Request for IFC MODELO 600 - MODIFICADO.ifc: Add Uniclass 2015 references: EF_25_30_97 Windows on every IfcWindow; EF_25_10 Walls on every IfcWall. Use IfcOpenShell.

First a look at what the model holds.

```python
import ifcopenshell

model = ifcopenshell.open("IFC MODELO 600 - MODIFICADO.ifc")
print(model.schema)
print("classifications:", [c.Name for c in model.by_type("IfcClassification")])
for ifc_class in ("IfcDoor", "IfcRoof", "IfcStair", "IfcWall", "IfcWindow"):
    print(ifc_class, len(model.by_type(ifc_class)))
```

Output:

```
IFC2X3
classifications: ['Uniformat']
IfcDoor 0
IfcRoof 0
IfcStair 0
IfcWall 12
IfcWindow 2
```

```python
import ifcopenshell
import ifcopenshell.api.classification

model = ifcopenshell.open("IFC MODELO 600 - MODIFICADO.ifc")

# IFC2X3 requires Source and Edition and has no link from the project to the system.
system = model.create_entity("IfcClassification", Source="NBS", Edition="2015", Name="Uniclass 2015")

codes = {
    "IfcWindow": ("EF_25_30_97", "Windows"),
    "IfcWall": ("EF_25_10", "Walls"),
}
for ifc_class, (code, name) in codes.items():
    products = model.by_type(ifc_class)
    ifcopenshell.api.classification.add_reference(
        model, products=products, classification=system, identification=code, name=name
    )
    print(code, len(products))

model.write("IFC MODELO 600 - MODIFICADO_updated.ifc")
```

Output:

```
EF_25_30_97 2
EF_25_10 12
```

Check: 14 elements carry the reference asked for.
